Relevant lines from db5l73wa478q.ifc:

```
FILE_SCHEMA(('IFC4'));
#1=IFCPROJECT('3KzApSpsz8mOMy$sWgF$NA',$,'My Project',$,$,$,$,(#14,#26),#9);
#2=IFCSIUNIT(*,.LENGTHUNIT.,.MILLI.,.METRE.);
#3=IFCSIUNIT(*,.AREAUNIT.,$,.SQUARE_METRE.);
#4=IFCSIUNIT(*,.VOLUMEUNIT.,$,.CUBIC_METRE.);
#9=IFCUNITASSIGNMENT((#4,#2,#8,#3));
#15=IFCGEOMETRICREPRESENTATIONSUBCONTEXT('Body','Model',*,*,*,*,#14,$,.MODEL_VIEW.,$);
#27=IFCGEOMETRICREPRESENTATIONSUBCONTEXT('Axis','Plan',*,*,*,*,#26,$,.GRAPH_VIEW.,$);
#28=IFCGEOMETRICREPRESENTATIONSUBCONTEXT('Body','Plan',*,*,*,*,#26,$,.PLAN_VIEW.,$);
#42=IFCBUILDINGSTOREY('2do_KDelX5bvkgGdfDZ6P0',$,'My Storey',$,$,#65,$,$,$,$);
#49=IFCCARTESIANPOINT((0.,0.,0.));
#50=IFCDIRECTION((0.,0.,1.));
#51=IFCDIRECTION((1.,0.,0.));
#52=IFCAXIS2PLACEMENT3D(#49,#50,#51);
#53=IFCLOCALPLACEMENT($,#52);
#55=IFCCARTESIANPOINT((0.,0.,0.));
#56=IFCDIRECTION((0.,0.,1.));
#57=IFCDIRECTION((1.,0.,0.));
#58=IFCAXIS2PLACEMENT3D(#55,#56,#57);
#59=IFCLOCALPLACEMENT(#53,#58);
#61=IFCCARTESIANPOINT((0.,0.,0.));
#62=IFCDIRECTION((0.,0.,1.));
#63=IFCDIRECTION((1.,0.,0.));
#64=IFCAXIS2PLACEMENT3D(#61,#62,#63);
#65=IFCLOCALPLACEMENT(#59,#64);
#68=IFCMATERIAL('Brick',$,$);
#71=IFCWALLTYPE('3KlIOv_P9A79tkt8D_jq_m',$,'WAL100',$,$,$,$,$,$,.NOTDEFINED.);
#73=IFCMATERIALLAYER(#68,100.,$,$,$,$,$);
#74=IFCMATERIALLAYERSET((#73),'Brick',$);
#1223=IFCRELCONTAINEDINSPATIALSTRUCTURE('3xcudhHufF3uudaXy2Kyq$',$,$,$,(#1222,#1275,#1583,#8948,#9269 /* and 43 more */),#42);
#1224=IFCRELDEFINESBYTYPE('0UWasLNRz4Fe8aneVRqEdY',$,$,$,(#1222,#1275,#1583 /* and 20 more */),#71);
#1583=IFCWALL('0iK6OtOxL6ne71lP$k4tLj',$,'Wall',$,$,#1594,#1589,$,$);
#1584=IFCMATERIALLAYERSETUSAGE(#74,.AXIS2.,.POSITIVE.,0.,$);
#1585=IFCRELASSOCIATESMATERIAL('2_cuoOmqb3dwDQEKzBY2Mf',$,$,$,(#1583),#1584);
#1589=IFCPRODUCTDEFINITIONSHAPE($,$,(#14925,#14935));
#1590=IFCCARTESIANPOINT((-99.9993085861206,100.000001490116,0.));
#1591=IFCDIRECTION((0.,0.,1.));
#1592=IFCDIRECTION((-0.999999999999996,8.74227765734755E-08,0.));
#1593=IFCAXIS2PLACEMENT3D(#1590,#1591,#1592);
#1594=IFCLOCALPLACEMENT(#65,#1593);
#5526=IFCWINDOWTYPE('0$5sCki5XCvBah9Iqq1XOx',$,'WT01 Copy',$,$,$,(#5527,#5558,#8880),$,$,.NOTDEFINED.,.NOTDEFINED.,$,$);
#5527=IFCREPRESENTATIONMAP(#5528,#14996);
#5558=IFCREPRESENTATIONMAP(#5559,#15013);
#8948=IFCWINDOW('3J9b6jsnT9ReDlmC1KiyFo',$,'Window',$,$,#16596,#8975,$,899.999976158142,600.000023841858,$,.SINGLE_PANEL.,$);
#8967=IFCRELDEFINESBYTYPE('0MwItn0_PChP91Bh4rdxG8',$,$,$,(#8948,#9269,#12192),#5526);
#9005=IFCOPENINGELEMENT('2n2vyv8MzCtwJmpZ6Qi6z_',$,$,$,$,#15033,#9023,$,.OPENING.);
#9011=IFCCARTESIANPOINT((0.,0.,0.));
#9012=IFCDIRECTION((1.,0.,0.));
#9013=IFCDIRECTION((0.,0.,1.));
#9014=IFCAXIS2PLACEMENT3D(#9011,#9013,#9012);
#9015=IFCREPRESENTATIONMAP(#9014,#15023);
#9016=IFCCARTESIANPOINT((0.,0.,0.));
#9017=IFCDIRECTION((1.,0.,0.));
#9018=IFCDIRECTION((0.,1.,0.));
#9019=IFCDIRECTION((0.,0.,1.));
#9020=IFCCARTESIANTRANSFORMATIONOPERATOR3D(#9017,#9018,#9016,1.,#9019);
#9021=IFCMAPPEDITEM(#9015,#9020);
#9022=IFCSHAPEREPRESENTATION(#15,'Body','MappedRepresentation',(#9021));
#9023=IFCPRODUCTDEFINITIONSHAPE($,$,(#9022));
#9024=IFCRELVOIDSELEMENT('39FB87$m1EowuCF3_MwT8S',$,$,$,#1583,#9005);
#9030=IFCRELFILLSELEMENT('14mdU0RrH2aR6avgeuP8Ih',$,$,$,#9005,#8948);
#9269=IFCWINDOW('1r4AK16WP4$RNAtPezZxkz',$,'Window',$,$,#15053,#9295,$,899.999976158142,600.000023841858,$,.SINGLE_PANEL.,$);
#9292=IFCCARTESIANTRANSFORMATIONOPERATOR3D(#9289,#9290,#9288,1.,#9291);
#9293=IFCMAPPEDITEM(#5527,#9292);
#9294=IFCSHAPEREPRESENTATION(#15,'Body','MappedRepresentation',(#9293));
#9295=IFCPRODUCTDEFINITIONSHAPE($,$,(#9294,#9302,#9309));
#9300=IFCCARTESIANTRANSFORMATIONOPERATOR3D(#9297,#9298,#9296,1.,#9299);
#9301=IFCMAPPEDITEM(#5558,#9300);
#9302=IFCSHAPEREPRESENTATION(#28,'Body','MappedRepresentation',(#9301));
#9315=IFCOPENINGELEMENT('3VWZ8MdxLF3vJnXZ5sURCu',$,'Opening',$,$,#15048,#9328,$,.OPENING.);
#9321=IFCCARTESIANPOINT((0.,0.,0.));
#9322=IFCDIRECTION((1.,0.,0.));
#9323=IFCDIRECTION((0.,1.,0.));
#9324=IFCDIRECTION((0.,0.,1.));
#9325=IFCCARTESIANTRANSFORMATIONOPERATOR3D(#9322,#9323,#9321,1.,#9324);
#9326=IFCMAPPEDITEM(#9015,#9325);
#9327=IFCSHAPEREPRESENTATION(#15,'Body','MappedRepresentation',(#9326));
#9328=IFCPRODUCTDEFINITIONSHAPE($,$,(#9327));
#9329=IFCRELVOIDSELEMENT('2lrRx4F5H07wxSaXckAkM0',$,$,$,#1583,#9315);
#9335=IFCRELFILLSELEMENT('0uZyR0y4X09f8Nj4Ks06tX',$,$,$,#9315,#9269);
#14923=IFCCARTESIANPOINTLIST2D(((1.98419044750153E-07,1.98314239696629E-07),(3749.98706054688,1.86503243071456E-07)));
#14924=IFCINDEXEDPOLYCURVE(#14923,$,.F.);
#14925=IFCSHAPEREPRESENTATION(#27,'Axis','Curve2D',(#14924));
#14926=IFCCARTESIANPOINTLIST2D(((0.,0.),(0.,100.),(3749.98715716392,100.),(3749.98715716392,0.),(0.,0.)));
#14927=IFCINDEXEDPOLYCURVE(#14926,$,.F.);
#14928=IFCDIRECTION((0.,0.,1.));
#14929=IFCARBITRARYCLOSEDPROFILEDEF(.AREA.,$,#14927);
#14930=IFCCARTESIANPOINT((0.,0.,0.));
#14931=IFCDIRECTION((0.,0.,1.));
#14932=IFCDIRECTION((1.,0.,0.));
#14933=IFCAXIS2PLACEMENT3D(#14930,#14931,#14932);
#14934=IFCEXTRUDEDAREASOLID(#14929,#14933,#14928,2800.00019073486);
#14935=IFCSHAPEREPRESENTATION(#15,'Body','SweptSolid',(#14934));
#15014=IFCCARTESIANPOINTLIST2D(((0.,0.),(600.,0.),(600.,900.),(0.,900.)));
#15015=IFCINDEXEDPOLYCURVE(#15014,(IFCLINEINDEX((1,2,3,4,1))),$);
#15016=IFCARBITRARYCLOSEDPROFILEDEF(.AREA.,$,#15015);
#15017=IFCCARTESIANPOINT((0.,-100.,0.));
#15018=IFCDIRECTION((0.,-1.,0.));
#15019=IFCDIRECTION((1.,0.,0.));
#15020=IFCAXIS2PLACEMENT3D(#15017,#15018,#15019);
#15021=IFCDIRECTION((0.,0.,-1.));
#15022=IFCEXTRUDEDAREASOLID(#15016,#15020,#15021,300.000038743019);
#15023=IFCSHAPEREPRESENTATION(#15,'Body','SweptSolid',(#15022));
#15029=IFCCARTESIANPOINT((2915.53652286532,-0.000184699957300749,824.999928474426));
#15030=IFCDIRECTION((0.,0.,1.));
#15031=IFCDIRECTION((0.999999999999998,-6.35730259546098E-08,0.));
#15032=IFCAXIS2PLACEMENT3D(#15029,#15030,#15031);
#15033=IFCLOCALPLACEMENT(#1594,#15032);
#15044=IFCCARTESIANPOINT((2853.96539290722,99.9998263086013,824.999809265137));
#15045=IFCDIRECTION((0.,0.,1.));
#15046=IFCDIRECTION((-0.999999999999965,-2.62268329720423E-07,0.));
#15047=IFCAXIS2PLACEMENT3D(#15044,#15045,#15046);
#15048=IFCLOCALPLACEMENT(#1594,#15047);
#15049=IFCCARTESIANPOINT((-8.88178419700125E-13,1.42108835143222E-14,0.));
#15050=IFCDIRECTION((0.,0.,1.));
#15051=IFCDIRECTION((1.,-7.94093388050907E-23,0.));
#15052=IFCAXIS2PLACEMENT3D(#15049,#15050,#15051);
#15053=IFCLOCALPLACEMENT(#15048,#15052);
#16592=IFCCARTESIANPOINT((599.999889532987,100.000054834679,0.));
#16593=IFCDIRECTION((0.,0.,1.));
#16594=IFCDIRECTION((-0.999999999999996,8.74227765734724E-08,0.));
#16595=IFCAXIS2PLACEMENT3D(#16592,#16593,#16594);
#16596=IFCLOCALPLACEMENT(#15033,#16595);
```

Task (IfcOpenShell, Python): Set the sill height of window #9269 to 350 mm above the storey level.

```python
import numpy as np
import ifcopenshell
import ifcopenshell.api.geometry
import ifcopenshell.geom
import ifcopenshell.util.element
import ifcopenshell.util.placement
import ifcopenshell.util.shape
import ifcopenshell.util.unit

model = ifcopenshell.open("db5l73wa478q.ifc")
unit_scale = ifcopenshell.util.unit.calculate_unit_scale(model)

window = model.by_id(9269)
opening = window.FillsVoids[0].RelatingOpeningElement
storey = ifcopenshell.util.element.get_container(window, ifc_class="IfcBuildingStorey")
level = ifcopenshell.util.placement.get_local_placement(storey.ObjectPlacement)[2, 3]

# The opening's origin need not be at the sill, so measure its lowest point.
shape = ifcopenshell.geom.create_shape(ifcopenshell.geom.settings(), opening)
bottom = ifcopenshell.util.shape.get_shape_bottom_elevation(shape, shape.geometry) / unit_scale
dz = level + 0.35 / unit_scale - bottom

shift = np.array([0.0, 0.0, dz])
# The window is placed relative to its opening, so it follows when the opening moves.
matrix = ifcopenshell.util.placement.get_local_placement(opening.ObjectPlacement)
matrix[:3, 3] += shift
ifcopenshell.api.geometry.edit_object_placement(
    model, product=opening, matrix=matrix, is_si=False, should_transform_children=True
)

print(f"moved by {dz * unit_scale:+.3f} m")

model.write("db5l73wa478q_rev.ifc")
```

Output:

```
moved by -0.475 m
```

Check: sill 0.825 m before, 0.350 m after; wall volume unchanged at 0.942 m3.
